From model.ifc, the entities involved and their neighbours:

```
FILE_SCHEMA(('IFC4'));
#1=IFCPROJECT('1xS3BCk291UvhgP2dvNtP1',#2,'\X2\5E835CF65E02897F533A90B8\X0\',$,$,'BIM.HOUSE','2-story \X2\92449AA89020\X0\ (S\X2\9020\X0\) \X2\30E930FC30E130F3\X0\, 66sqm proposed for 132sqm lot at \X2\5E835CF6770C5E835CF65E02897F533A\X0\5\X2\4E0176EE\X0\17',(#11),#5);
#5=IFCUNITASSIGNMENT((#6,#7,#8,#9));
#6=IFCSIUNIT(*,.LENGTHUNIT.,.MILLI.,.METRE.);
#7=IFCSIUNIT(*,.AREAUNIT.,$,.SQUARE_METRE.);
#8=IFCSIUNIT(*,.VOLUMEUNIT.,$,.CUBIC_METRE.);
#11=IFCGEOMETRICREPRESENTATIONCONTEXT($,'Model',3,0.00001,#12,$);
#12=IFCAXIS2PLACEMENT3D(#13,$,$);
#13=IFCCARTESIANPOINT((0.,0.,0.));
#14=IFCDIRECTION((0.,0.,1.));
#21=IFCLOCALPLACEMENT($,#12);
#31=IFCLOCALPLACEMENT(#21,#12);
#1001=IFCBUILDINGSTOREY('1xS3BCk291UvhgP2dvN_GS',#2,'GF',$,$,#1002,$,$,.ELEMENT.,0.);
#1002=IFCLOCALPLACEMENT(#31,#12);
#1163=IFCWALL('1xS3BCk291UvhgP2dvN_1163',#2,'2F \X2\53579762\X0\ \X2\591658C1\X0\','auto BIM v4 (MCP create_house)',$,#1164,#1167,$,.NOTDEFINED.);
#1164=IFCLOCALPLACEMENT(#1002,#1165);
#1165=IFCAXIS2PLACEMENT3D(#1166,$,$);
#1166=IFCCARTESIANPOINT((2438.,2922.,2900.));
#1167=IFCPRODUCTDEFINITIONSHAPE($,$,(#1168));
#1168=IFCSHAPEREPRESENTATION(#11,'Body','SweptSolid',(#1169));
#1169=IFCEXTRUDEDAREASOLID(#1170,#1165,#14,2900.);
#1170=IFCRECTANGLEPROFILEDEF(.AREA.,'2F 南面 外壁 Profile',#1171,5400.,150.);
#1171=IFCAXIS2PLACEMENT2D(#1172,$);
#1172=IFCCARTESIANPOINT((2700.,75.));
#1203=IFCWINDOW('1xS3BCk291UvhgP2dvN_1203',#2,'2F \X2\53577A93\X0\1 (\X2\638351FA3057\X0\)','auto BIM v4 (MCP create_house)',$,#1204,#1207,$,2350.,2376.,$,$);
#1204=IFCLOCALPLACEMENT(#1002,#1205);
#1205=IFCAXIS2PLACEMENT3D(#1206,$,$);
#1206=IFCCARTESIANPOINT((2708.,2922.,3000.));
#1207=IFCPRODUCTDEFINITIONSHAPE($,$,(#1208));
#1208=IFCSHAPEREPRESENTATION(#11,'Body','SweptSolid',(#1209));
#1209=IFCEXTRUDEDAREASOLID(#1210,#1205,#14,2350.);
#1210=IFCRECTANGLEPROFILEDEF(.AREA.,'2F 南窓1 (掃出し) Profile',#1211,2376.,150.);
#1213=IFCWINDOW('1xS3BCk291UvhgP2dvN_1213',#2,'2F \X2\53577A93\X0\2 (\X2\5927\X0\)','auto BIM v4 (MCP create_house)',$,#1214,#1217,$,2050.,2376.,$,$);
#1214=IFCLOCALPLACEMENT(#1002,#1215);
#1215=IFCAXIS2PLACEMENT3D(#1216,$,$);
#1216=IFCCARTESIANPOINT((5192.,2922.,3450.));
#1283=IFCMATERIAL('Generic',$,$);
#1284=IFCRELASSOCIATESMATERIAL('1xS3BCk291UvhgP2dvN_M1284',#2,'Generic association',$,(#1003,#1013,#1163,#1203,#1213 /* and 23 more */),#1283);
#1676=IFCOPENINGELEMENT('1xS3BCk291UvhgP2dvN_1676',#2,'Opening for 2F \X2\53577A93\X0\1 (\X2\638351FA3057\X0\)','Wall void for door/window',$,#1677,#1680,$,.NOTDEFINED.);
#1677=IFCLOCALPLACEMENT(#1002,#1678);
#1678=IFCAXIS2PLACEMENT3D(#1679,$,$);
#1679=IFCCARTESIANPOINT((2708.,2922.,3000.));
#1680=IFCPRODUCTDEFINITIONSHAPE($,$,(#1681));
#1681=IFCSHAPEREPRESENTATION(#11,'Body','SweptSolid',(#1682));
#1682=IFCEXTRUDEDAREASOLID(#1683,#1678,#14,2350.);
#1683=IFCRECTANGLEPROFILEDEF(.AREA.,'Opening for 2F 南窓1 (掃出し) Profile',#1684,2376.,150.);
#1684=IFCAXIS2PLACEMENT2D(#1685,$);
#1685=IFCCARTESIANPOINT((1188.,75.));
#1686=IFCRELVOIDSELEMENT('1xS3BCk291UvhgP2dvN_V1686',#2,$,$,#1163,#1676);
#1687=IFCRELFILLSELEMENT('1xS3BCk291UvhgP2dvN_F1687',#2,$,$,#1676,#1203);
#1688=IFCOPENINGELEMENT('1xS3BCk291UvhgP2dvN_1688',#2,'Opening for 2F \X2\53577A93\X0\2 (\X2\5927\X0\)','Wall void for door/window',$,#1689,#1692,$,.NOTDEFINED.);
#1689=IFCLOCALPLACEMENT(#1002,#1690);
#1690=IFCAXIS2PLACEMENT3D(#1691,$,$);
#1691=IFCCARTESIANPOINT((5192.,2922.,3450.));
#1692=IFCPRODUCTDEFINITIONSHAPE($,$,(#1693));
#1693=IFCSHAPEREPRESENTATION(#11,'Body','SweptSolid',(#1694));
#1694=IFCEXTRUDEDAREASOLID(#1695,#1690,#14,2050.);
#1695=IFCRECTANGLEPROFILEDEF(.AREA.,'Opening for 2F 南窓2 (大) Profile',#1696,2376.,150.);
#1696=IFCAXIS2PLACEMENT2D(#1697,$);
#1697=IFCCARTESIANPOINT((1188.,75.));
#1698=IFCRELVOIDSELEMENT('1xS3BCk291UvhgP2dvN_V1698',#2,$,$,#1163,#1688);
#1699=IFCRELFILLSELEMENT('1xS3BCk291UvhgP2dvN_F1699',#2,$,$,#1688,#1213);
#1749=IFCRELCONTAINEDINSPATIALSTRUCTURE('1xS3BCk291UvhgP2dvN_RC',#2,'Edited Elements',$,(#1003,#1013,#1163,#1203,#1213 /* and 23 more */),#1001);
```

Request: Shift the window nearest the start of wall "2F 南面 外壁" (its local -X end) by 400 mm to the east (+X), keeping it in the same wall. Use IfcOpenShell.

```python
import ifcopenshell
import ifcopenshell.api.geometry
import ifcopenshell.util.placement
import ifcopenshell.util.unit

model = ifcopenshell.open("model.ifc")
unit_scale = ifcopenshell.util.unit.calculate_unit_scale(model)

window = model.by_guid("1xS3BCk291UvhgP2dvN_1203")
opening = window.FillsVoids[0].RelatingOpeningElement
wall = opening.VoidsElements[0].RelatingBuildingElement

wall_matrix = ifcopenshell.util.placement.get_local_placement(wall.ObjectPlacement)
shift = wall_matrix[:3, 0] * 0.4 / unit_scale
before = ifcopenshell.util.placement.get_local_placement(window.ObjectPlacement)[:3, 3].copy()

# The window is not placed relative to its opening, so move both.
for product in (opening, window):
    matrix = ifcopenshell.util.placement.get_local_placement(product.ObjectPlacement)
    matrix[:3, 3] += shift
    ifcopenshell.api.geometry.edit_object_placement(model, product=product, matrix=matrix, is_si=False)

after = ifcopenshell.util.placement.get_local_placement(window.ObjectPlacement)[:3, 3]
print("window moved by", (after - before).round(3) + 0.0)

model.write("model_rev.ifc")
```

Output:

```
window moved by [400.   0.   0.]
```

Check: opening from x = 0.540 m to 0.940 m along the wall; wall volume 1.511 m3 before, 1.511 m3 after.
